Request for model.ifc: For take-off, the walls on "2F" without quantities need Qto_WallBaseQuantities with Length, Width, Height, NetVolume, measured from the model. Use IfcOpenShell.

First a look at what the model holds.

```python
import ifcopenshell
import ifcopenshell.util.element
import ifcopenshell.util.unit

model = ifcopenshell.open("model.ifc")
print(model.schema)
for unit_type in ("LENGTHUNIT", "AREAUNIT", "VOLUMEUNIT"):
    print(unit_type, ifcopenshell.util.unit.calculate_unit_scale(model, unit_type))
storey = next(s for s in model.by_type("IfcBuildingStorey") if s.Name == "2F")
walls = [e for e in ifcopenshell.util.element.get_decomposition(storey) if e.is_a("IfcWall")]
for e in sorted(walls, key=lambda e: e.id()):
    print(e.id(), e.is_a(), e.Name, list(ifcopenshell.util.element.get_psets(e, qtos_only=True)), sep=" | ")
```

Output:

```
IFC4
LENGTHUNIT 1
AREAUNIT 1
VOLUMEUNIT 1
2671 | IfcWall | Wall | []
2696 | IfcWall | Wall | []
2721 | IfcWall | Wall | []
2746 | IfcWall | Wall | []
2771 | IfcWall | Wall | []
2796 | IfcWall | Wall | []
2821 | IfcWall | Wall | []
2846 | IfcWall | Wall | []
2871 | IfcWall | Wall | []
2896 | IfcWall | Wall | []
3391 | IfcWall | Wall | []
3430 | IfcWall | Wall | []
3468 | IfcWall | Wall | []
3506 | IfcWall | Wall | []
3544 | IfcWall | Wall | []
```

```python
import ifcopenshell
import ifcopenshell.api.pset
import ifcopenshell.geom
import ifcopenshell.util.element
import ifcopenshell.util.shape
import ifcopenshell.util.unit

model = ifcopenshell.open("model.ifc")
unit_scale = ifcopenshell.util.unit.calculate_unit_scale(model)
volume_scale = ifcopenshell.util.unit.calculate_unit_scale(model, "VOLUMEUNIT")
settings = ifcopenshell.geom.settings()

storey = next(s for s in model.by_type("IfcBuildingStorey") if s.Name == "2F")
walls = [e for e in ifcopenshell.util.element.get_decomposition(storey) if e.is_a("IfcWall")]

for e in sorted(walls, key=lambda e: e.id()):
    if ifcopenshell.util.element.get_psets(e, qtos_only=True, should_inherit=False):
        continue
    # Geometry comes back in metres, in the element's own axes.
    shape = ifcopenshell.geom.create_shape(settings, e)
    values = {
        "Length": ifcopenshell.util.shape.get_x(shape.geometry) / unit_scale,
        "Width": ifcopenshell.util.shape.get_y(shape.geometry) / unit_scale,
        "Height": ifcopenshell.util.shape.get_z(shape.geometry) / unit_scale,
        "NetVolume": ifcopenshell.util.shape.get_volume(shape.geometry) / volume_scale,
    }
    qto = ifcopenshell.api.pset.add_qto(model, product=e, name="Qto_WallBaseQuantities")
    ifcopenshell.api.pset.edit_qto(model, qto=qto, properties=values)
    print(e.id(), {k: round(v, 3) for k, v in values.items()})

model.write("model_updated.ifc")
```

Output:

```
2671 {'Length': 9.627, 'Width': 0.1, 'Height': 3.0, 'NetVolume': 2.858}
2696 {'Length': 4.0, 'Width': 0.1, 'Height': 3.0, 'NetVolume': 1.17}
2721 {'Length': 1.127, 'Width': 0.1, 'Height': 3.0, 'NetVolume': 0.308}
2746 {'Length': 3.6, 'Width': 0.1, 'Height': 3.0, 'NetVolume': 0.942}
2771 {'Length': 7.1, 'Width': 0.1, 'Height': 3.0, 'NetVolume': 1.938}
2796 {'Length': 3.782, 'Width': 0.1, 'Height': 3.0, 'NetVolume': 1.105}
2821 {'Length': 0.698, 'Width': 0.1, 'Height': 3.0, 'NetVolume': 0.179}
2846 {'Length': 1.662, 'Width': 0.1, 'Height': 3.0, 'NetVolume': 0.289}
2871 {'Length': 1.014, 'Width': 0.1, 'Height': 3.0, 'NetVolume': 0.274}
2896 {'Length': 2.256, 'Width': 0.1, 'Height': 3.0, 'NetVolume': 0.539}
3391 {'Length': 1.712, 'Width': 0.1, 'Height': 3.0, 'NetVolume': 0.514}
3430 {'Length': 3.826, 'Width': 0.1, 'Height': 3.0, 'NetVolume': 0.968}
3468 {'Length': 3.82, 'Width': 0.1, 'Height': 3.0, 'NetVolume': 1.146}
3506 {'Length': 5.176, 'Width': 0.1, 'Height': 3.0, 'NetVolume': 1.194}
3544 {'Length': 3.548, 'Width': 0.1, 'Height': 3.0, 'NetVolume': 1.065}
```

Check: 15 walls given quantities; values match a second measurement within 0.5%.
